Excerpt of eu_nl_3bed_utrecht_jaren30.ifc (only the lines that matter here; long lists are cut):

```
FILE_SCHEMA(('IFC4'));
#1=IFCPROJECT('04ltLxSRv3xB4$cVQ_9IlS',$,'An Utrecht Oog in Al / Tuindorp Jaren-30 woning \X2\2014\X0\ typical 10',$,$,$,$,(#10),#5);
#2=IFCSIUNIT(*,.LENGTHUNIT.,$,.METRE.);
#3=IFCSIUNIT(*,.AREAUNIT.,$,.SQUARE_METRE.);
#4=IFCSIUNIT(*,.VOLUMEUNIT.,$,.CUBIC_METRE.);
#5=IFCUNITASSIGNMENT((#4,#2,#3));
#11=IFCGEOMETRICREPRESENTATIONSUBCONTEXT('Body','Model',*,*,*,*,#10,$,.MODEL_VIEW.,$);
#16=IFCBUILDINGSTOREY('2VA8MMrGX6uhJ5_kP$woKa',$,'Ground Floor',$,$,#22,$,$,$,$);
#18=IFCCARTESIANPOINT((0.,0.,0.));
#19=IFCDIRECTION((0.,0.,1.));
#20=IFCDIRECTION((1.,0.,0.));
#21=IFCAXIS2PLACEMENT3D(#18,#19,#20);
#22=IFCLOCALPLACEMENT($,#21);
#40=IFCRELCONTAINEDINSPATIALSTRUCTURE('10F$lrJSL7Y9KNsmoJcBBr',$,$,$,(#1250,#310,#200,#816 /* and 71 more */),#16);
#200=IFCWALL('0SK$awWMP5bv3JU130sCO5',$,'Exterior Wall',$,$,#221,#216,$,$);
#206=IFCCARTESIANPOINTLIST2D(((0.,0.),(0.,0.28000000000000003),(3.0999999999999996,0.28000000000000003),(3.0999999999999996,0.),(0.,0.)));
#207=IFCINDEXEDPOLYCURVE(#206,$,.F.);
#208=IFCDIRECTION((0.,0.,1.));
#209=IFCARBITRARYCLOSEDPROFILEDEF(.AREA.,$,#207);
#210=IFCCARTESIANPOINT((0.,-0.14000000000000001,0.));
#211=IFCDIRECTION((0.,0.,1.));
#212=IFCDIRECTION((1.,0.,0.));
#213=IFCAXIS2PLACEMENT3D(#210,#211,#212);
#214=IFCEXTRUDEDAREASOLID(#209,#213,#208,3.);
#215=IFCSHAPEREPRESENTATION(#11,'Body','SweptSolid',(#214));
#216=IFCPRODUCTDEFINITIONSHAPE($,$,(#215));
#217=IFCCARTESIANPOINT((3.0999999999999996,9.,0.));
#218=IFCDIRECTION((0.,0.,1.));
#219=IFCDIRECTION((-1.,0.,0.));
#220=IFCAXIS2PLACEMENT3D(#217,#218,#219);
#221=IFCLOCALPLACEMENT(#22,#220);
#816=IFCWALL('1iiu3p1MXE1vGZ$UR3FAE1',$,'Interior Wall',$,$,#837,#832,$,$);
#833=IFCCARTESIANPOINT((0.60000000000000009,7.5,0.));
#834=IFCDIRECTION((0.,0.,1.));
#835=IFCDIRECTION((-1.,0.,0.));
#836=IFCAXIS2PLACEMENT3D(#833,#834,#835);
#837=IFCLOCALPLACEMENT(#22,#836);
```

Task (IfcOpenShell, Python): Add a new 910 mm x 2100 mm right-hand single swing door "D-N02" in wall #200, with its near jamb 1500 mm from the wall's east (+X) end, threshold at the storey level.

```python
import numpy as np
import ifcopenshell
import ifcopenshell.api.feature
import ifcopenshell.api.geometry
import ifcopenshell.api.root
import ifcopenshell.api.spatial
import ifcopenshell.geom
import ifcopenshell.util.element
import ifcopenshell.util.placement
import ifcopenshell.util.representation
import ifcopenshell.util.shape
import ifcopenshell.util.unit

model = ifcopenshell.open("eu_nl_3bed_utrecht_jaren30.ifc")
unit_scale = ifcopenshell.util.unit.calculate_unit_scale(model)
settings = ifcopenshell.geom.settings()


def volume(element):
    """Net volume in cubic metres, openings subtracted."""
    shape = ifcopenshell.geom.create_shape(settings, element)
    return ifcopenshell.util.shape.get_volume(shape.geometry)


wall = model.by_guid("0SK$awWMP5bv3JU130sCO5")
storey = ifcopenshell.util.element.get_container(wall, ifc_class="IfcBuildingStorey")
context = ifcopenshell.util.representation.get_context(model, "Model", "Body", "MODEL_VIEW")
before = volume(wall)

width, height, from_end, sill = 0.91, 2.1, 1.5, 0.0  # metres

# The wall runs along its own X axis, and the end named is its -X end.
wall_shape = ifcopenshell.geom.create_shape(settings, wall)
x, y, z = ifcopenshell.util.shape.get_vertices(wall_shape.geometry).T
start = x.min() + from_end
face, thickness = float(y.min()), float(y.max() - y.min())
wall_matrix = ifcopenshell.util.placement.get_local_placement(wall.ObjectPlacement)
level = ifcopenshell.util.placement.get_local_placement(storey.ObjectPlacement)[2, 3]


def in_wall(x, y):
    """Placement at x, y metres in the wall's axes, at sill height."""
    matrix = wall_matrix.copy()
    matrix[:, 3] = wall_matrix @ np.array([x / unit_scale, y / unit_scale, 0.0, 1.0])
    matrix[2, 3] = level + sill / unit_scale
    return matrix


# Opening: a box that overshoots both wall faces by 50 mm.
opening = ifcopenshell.api.root.create_entity(model, ifc_class="IfcOpeningElement", predefined_type="OPENING")
box = ifcopenshell.api.geometry.add_wall_representation(
    model, context=context, length=width, height=height, thickness=thickness + 0.1
)
ifcopenshell.api.geometry.assign_representation(model, product=opening, representation=box)
ifcopenshell.api.geometry.edit_object_placement(model, product=opening, matrix=in_wall(start, face - 0.05), is_si=False)
ifcopenshell.api.feature.add_feature(model, feature=opening, element=wall)

door = ifcopenshell.api.root.create_entity(model, ifc_class="IfcDoor", name="D-N02", predefined_type="DOOR")
door.OverallWidth, door.OverallHeight = width / unit_scale, height / unit_scale
door.OperationType = "SINGLE_SWING_RIGHT"
body = ifcopenshell.api.geometry.add_door_representation(
    model,
    context=context,
    overall_width=door.OverallWidth,
    overall_height=door.OverallHeight,
    operation_type="SINGLE_SWING_RIGHT",
    lining_properties={"LiningDepth": thickness / unit_scale, "ThresholdDepth": thickness / unit_scale},
)
ifcopenshell.api.geometry.assign_representation(model, product=door, representation=body)
ifcopenshell.api.spatial.assign_container(model, products=[door], relating_structure=storey)
ifcopenshell.api.feature.add_filling(model, opening=opening, element=door)

# The lining spans the wall, so the door starts at the wall face.
ifcopenshell.api.geometry.edit_object_placement(model, product=door, matrix=in_wall(start, face), is_si=False)

after = volume(wall)

print(f"wall volume {before:.3f} -> {after:.3f} m3")

model.write("eu_nl_3bed_utrecht_jaren30_rev.ifc")
```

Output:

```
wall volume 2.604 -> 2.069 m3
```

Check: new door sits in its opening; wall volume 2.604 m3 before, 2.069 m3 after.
